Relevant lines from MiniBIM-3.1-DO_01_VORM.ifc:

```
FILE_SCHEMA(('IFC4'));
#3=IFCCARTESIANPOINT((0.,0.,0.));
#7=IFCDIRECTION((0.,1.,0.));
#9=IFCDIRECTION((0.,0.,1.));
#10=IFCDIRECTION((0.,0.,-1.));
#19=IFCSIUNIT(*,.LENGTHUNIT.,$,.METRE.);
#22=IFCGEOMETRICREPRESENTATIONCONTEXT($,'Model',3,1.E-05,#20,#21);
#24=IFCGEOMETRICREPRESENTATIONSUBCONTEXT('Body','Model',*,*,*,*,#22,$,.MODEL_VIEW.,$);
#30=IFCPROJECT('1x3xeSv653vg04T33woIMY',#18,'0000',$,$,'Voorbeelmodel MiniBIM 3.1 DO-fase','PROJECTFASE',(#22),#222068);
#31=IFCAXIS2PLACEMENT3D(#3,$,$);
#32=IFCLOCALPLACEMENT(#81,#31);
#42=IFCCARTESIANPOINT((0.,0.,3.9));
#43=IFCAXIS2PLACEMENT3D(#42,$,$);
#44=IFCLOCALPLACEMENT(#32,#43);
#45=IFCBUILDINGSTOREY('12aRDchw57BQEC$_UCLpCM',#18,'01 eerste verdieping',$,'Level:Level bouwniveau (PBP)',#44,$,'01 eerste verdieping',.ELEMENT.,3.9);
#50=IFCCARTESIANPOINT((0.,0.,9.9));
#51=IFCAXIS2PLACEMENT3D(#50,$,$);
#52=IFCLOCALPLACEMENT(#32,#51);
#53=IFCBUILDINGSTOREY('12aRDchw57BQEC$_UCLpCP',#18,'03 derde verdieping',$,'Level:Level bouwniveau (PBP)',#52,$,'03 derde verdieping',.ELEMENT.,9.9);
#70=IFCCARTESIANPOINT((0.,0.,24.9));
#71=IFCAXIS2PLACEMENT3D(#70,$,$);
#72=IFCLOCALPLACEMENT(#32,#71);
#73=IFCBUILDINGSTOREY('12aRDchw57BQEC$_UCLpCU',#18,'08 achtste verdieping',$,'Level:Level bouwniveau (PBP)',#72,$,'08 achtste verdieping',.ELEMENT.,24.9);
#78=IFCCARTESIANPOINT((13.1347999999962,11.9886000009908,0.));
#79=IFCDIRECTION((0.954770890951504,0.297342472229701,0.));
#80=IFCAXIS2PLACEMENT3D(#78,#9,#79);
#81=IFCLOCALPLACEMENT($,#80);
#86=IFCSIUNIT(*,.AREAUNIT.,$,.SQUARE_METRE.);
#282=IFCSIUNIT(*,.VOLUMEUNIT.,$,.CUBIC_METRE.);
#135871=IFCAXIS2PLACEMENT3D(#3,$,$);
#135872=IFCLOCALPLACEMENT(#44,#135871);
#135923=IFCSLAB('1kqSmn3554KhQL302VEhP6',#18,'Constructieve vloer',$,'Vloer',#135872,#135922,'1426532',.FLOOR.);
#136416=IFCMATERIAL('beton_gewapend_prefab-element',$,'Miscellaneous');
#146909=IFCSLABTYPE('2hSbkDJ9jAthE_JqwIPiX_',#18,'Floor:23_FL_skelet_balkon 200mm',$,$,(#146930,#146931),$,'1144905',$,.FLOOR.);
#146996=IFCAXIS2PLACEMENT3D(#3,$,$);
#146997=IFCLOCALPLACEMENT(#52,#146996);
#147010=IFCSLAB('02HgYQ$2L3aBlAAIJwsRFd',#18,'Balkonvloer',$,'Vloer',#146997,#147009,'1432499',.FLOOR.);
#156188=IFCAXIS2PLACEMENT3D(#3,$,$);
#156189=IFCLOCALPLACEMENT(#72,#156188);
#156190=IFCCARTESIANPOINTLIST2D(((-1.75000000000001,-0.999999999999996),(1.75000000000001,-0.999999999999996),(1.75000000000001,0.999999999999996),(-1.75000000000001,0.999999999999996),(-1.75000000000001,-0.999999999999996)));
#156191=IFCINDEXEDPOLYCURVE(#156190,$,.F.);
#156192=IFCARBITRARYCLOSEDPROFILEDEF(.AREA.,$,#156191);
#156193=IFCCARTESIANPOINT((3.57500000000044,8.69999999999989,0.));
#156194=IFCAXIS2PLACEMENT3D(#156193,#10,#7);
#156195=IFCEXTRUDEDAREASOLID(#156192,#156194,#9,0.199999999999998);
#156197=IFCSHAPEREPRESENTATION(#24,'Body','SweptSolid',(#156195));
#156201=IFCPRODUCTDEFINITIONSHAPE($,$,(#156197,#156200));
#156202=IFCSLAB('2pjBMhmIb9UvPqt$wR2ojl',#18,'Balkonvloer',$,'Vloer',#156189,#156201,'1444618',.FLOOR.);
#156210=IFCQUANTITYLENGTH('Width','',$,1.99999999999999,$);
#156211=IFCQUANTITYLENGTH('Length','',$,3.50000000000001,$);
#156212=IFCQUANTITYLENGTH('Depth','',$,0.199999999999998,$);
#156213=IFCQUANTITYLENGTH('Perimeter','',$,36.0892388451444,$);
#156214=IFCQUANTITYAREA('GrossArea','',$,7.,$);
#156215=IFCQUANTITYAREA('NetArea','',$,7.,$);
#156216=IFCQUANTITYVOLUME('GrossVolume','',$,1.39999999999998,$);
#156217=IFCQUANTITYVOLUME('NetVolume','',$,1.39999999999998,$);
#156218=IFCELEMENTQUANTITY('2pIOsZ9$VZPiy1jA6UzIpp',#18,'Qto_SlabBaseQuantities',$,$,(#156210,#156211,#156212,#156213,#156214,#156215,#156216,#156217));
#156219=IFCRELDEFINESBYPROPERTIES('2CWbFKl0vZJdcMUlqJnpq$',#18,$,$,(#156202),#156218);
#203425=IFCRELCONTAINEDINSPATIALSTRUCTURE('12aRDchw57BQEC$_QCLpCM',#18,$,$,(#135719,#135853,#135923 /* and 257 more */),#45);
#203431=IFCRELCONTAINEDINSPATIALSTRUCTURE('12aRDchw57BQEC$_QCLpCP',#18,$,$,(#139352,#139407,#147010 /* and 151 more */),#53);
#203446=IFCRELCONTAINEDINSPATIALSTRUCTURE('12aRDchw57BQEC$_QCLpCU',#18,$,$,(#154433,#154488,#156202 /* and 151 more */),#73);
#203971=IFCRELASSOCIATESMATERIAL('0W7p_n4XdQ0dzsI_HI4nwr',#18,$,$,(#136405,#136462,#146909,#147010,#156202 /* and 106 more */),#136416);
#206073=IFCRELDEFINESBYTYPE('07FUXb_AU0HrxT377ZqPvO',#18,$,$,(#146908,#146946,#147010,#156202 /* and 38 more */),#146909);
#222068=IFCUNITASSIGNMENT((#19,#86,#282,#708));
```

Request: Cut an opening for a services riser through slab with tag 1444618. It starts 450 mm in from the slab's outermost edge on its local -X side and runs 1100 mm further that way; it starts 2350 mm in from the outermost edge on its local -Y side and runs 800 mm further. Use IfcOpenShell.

```python
import numpy as np
import ifcopenshell
import ifcopenshell.api.feature
import ifcopenshell.api.geometry
import ifcopenshell.api.pset
import ifcopenshell.api.root
import ifcopenshell.geom
import ifcopenshell.util.element
import ifcopenshell.util.placement
import ifcopenshell.util.representation
import ifcopenshell.util.shape
import ifcopenshell.util.unit

model = ifcopenshell.open("MiniBIM-3.1-DO_01_VORM.ifc")
unit_scale = ifcopenshell.util.unit.calculate_unit_scale(model)
area_scale = ifcopenshell.util.unit.calculate_unit_scale(model, "AREAUNIT")
volume_scale = ifcopenshell.util.unit.calculate_unit_scale(model, "VOLUMEUNIT")
settings = ifcopenshell.geom.settings()


def volume(element):
    """Net volume in cubic metres, openings subtracted."""
    shape = ifcopenshell.geom.create_shape(settings, element)
    return ifcopenshell.util.shape.get_volume(shape.geometry)


slab = model.by_id(156202)
before = volume(slab)

# Extent in the slab's own axes, in metres. The edges named are its -X and -Y sides.
slab_shape = ifcopenshell.geom.create_shape(settings, slab)
vertices = ifcopenshell.util.shape.get_vertices(slab_shape.geometry)
x_min, y_min, bottom = vertices.min(axis=0)
top = vertices[:, 2].max()

opening = ifcopenshell.api.root.create_entity(model, ifc_class="IfcOpeningElement", name="Services riser opening", predefined_type="OPENING")
context = ifcopenshell.util.representation.get_context(model, "Model", "Body", "MODEL_VIEW")
width, depth = 1.1, 0.8
outline = [(0.0, 0.0), (width, 0.0), (width, depth), (0.0, depth), (0.0, 0.0)]
# Overshoot both faces by 50 mm so the cut is clean.
shape = ifcopenshell.api.geometry.add_slab_representation(
    model, context=context, depth=top - bottom + 0.1, polyline=outline
)
ifcopenshell.api.geometry.assign_representation(model, product=opening, representation=shape)

matrix = ifcopenshell.util.placement.get_local_placement(slab.ObjectPlacement)
matrix[:, 3] = matrix @ np.append(np.array([x_min + 0.45, y_min + 2.35, bottom - 0.05]) / unit_scale, 1.0)
ifcopenshell.api.geometry.edit_object_placement(model, product=opening, matrix=matrix, is_si=False)
ifcopenshell.api.feature.add_feature(model, feature=opening, element=slab)

after = volume(slab)

# Update the slab's stored quantities.
qto = model.by_id(ifcopenshell.util.element.get_pset(slab, "Qto_SlabBaseQuantities", should_inherit=False)["id"])
ifcopenshell.api.pset.edit_qto(model, qto=qto, properties={
    "NetArea": after / (top - bottom) / area_scale,
    "NetVolume": after / volume_scale,
})

print(f"slab volume {before:.3f} -> {after:.3f} m3")

model.write("MiniBIM-3.1-DO_01_VORM-out.ifc")
```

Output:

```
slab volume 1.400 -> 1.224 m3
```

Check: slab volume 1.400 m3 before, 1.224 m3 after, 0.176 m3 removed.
